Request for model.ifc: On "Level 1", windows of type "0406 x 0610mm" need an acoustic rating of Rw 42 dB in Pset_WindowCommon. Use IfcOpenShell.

First a look at what the model holds.

```python
import ifcopenshell
import ifcopenshell.util.element

model = ifcopenshell.open("model.ifc")
print(model.schema)
storey = next(s for s in model.by_type("IfcBuildingStorey") if s.Name == "Level 1")
windows = [e for e in ifcopenshell.util.element.get_decomposition(storey) if e.is_a("IfcWindow")]
seen = {}
for e in windows:
    element_type = ifcopenshell.util.element.get_type(e)
    key = (element_type.Name if element_type != e and element_type else None, ifcopenshell.util.element.get_pset(e, "Pset_WindowCommon", "AcousticRating"))
    seen[key] = seen.get(key, 0) + 1
for (name, value), count in sorted(seen.items(), key=str):
    print(count, "x", name, "|", value)
```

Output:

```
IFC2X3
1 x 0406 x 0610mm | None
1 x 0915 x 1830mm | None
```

```python
import ifcopenshell
import ifcopenshell.api.pset
import ifcopenshell.util.element

model = ifcopenshell.open("model.ifc")

storey = next(s for s in model.by_type("IfcBuildingStorey") if s.Name == "Level 1")
windows = [e for e in ifcopenshell.util.element.get_decomposition(storey) if e.is_a("IfcWindow")]

count = 0
for e in windows:
    element_type = ifcopenshell.util.element.get_type(e)
    if element_type in (None, e) or element_type.Name != "0406 x 0610mm":
        continue
    # add_pset returns the element's existing set when there is one.
    pset = ifcopenshell.api.pset.add_pset(model, product=e, name="Pset_WindowCommon")
    ifcopenshell.api.pset.edit_pset(model, pset=pset, properties={"AcousticRating": "Rw 42 dB"})
    count += 1

print(count, "windows updated")

model.write("model_updated.ifc")
```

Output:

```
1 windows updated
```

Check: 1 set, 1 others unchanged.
